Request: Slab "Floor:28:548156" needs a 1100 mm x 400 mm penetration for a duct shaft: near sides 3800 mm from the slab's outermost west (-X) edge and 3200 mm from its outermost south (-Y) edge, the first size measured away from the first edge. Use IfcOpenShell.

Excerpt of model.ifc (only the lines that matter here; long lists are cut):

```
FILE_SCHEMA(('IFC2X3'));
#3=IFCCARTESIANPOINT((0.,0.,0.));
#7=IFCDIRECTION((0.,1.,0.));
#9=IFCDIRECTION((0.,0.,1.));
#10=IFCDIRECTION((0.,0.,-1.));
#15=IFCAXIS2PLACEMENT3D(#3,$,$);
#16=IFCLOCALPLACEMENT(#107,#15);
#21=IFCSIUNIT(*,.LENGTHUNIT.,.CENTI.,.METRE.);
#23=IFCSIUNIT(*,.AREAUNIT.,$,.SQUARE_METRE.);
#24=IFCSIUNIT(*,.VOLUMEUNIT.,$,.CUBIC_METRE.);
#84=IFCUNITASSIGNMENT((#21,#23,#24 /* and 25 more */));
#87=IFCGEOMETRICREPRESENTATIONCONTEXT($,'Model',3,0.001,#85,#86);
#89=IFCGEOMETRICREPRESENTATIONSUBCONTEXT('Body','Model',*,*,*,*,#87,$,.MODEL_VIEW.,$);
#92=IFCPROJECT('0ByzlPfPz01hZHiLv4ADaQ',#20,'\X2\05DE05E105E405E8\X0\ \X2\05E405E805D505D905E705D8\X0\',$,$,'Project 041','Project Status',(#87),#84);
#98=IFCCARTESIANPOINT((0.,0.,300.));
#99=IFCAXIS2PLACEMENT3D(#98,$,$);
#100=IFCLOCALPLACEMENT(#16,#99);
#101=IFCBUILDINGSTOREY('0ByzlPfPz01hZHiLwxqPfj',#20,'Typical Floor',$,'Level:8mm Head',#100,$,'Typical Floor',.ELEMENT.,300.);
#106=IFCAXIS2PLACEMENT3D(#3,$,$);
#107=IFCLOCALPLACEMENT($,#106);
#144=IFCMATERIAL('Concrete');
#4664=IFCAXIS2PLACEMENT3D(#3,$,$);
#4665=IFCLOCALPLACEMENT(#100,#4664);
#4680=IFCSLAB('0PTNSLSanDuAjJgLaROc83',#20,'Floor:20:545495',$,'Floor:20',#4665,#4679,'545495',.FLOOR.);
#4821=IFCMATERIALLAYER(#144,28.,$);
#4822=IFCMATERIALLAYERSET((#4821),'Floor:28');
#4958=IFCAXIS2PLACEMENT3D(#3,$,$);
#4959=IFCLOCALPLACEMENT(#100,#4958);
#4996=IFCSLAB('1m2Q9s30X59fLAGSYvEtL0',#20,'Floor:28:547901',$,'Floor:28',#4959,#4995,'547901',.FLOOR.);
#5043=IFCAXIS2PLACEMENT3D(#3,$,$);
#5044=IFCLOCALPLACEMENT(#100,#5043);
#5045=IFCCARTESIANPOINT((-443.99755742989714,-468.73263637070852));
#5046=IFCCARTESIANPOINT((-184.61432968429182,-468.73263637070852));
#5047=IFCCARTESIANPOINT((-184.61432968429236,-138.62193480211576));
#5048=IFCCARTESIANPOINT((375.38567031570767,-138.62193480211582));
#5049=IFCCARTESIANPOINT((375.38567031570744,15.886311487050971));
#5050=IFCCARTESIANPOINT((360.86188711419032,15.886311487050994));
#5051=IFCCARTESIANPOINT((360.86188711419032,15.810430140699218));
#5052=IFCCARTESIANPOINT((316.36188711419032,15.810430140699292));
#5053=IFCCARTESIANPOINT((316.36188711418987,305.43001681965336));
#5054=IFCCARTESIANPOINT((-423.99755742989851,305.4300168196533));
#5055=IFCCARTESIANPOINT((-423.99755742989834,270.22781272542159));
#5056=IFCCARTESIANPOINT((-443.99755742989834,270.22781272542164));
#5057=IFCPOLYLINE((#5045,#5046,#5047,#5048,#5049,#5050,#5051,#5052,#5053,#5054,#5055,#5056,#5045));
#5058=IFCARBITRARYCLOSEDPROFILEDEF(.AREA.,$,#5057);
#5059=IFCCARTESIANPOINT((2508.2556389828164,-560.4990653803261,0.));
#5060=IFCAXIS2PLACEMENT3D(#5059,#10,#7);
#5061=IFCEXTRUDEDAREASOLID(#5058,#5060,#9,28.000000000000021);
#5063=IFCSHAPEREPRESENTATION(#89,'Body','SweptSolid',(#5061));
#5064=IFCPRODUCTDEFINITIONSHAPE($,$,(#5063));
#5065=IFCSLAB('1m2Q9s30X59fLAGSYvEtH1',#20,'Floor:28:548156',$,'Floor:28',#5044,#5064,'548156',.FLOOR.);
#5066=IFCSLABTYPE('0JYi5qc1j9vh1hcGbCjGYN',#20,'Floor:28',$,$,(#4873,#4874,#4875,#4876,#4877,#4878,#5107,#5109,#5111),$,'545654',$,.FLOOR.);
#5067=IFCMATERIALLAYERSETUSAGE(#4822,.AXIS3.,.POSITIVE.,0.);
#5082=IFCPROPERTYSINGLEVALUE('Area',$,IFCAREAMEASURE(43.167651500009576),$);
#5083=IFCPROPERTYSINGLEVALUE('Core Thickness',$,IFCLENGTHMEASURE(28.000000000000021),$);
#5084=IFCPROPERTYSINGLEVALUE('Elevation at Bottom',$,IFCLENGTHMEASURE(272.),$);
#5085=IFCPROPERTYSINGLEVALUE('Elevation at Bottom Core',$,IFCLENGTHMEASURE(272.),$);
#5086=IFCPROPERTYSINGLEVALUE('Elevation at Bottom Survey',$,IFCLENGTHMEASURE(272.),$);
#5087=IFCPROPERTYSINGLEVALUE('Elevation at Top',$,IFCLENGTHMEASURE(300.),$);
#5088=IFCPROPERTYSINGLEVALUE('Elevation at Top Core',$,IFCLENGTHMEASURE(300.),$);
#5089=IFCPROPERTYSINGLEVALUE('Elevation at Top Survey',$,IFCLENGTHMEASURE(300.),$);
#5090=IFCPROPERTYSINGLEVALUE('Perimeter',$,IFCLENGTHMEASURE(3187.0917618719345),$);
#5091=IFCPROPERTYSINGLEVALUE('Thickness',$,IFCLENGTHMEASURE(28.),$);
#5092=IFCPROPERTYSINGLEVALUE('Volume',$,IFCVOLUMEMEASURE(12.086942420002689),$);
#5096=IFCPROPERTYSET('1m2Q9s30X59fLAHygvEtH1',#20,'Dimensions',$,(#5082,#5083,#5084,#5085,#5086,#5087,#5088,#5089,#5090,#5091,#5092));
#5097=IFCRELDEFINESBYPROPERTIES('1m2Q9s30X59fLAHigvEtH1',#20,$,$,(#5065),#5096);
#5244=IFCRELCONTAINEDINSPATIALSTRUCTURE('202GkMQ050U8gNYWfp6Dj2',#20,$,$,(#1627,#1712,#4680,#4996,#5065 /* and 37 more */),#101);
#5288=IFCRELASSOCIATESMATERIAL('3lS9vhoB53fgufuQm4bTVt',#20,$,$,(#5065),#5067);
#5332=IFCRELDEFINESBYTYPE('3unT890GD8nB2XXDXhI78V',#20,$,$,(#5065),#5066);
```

```python
import numpy as np
import ifcopenshell
import ifcopenshell.api.feature
import ifcopenshell.api.geometry
import ifcopenshell.api.pset
import ifcopenshell.api.root
import ifcopenshell.geom
import ifcopenshell.util.element
import ifcopenshell.util.placement
import ifcopenshell.util.representation
import ifcopenshell.util.shape
import ifcopenshell.util.unit

model = ifcopenshell.open("model.ifc")
unit_scale = ifcopenshell.util.unit.calculate_unit_scale(model)
area_scale = ifcopenshell.util.unit.calculate_unit_scale(model, "AREAUNIT")
volume_scale = ifcopenshell.util.unit.calculate_unit_scale(model, "VOLUMEUNIT")
settings = ifcopenshell.geom.settings()


def volume(element):
    """Net volume in cubic metres, openings subtracted."""
    shape = ifcopenshell.geom.create_shape(settings, element)
    return ifcopenshell.util.shape.get_volume(shape.geometry)


slab = model.by_guid("1m2Q9s30X59fLAGSYvEtH1")
before = volume(slab)

# Extent in the slab's own axes, in metres. The edges named are its -X and -Y sides.
slab_shape = ifcopenshell.geom.create_shape(settings, slab)
vertices = ifcopenshell.util.shape.get_vertices(slab_shape.geometry)
x_min, y_min, bottom = vertices.min(axis=0)
top = vertices[:, 2].max()

opening = ifcopenshell.api.root.create_entity(model, ifc_class="IfcOpeningElement", name="Duct shaft opening")
context = ifcopenshell.util.representation.get_context(model, "Model", "Body", "MODEL_VIEW")
width, depth = 1.1, 0.4
outline = [(0.0, 0.0), (width, 0.0), (width, depth), (0.0, depth), (0.0, 0.0)]
# Overshoot both faces by 50 mm so the cut is clean.
shape = ifcopenshell.api.geometry.add_slab_representation(
    model, context=context, depth=top - bottom + 0.1, polyline=outline
)
ifcopenshell.api.geometry.assign_representation(model, product=opening, representation=shape)

matrix = ifcopenshell.util.placement.get_local_placement(slab.ObjectPlacement)
matrix[:, 3] = matrix @ np.append(np.array([x_min + 3.8, y_min + 3.2, bottom - 0.05]) / unit_scale, 1.0)
ifcopenshell.api.geometry.edit_object_placement(model, product=opening, matrix=matrix, is_si=False)
ifcopenshell.api.feature.add_feature(model, feature=opening, element=slab)

after = volume(slab)

# Update the slab's stored quantities.
pset = model.by_id(ifcopenshell.util.element.get_pset(slab, "Dimensions", should_inherit=False)["id"])
ifcopenshell.api.pset.edit_pset(model, pset=pset, properties={
    "Area": model.create_entity("IfcAreaMeasure", after / (top - bottom) / area_scale),
    "Volume": model.create_entity("IfcVolumeMeasure", after / volume_scale),
})

print(f"slab volume {before:.3f} -> {after:.3f} m3")

model.write("model_edited.ifc")
```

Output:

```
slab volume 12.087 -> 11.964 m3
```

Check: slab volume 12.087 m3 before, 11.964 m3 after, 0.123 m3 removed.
